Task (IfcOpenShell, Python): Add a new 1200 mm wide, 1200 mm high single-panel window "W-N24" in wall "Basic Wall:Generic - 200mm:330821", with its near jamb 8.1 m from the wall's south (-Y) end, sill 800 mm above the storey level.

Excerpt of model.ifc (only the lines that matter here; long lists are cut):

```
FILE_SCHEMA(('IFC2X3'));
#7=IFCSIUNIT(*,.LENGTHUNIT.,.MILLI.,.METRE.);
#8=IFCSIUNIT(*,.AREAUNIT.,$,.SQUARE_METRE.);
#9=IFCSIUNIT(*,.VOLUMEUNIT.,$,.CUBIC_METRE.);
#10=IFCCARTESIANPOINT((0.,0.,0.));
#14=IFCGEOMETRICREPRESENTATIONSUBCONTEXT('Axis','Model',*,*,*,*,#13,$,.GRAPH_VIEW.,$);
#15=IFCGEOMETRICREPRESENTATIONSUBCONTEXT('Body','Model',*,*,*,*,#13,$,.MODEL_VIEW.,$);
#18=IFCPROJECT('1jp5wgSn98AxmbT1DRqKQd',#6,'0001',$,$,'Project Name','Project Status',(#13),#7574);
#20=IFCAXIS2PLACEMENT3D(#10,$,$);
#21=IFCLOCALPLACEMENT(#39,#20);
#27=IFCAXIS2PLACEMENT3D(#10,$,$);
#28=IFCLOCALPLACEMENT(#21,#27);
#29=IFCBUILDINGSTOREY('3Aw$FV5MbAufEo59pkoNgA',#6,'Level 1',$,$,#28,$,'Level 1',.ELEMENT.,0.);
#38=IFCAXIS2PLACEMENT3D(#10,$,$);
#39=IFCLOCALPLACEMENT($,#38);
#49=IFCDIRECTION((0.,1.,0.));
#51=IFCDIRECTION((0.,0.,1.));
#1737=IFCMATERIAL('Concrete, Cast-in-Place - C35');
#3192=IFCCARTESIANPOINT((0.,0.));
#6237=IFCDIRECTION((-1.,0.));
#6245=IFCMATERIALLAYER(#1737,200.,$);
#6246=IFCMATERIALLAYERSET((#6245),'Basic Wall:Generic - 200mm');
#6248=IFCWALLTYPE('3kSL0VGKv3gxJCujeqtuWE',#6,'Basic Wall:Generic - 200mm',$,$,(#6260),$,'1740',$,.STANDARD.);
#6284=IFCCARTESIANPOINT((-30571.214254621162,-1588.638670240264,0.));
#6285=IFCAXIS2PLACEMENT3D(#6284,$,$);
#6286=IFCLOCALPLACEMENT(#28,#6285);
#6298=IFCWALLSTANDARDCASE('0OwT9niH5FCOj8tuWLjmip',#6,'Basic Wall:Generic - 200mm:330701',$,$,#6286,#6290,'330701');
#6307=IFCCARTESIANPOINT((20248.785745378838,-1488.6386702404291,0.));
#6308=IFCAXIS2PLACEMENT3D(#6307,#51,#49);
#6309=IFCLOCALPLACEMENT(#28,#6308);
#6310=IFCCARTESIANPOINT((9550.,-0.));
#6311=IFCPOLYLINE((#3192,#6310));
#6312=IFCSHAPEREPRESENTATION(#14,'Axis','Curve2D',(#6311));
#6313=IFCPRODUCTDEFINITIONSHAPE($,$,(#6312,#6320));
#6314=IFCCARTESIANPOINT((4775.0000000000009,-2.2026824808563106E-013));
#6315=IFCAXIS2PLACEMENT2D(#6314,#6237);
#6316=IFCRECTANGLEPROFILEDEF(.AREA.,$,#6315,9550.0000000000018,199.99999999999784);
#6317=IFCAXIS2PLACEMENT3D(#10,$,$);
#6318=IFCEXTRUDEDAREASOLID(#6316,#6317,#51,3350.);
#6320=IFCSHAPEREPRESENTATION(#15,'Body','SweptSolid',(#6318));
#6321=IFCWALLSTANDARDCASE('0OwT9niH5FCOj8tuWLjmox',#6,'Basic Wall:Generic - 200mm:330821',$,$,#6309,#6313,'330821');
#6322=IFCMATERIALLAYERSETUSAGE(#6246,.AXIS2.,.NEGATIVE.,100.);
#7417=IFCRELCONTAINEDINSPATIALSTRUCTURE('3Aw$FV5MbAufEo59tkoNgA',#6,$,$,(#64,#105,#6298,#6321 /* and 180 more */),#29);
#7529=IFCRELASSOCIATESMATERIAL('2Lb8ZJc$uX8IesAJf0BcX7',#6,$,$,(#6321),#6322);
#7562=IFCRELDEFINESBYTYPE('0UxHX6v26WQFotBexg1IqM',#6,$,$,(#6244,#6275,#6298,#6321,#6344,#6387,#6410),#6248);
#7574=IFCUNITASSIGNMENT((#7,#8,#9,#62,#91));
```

```python
import numpy as np
import ifcopenshell
import ifcopenshell.api.feature
import ifcopenshell.api.geometry
import ifcopenshell.api.root
import ifcopenshell.api.spatial
import ifcopenshell.api.type
import ifcopenshell.geom
import ifcopenshell.util.element
import ifcopenshell.util.placement
import ifcopenshell.util.representation
import ifcopenshell.util.shape
import ifcopenshell.util.unit

model = ifcopenshell.open("model.ifc")
unit_scale = ifcopenshell.util.unit.calculate_unit_scale(model)
settings = ifcopenshell.geom.settings()


def volume(element):
    """Net volume in cubic metres, openings subtracted."""
    shape = ifcopenshell.geom.create_shape(settings, element)
    return ifcopenshell.util.shape.get_volume(shape.geometry)


wall = model.by_guid("0OwT9niH5FCOj8tuWLjmox")
storey = ifcopenshell.util.element.get_container(wall, ifc_class="IfcBuildingStorey")
context = ifcopenshell.util.representation.get_context(model, "Model", "Body", "MODEL_VIEW")
before = volume(wall)

width, height, from_end, sill = 1.2, 1.2, 8.1, 0.8  # metres

# The wall runs along its own X axis, and the end named is its -X end.
wall_shape = ifcopenshell.geom.create_shape(settings, wall)
x, y, z = ifcopenshell.util.shape.get_vertices(wall_shape.geometry).T
start = x.min() + from_end
face, thickness = float(y.min()), float(y.max() - y.min())
wall_matrix = ifcopenshell.util.placement.get_local_placement(wall.ObjectPlacement)
level = ifcopenshell.util.placement.get_local_placement(storey.ObjectPlacement)[2, 3]


def in_wall(x, y):
    """Placement at x, y metres in the wall's axes, at sill height."""
    matrix = wall_matrix.copy()
    matrix[:, 3] = wall_matrix @ np.array([x / unit_scale, y / unit_scale, 0.0, 1.0])
    matrix[2, 3] = level + sill / unit_scale
    return matrix


# Opening: a box that overshoots both wall faces by 50 mm.
opening = ifcopenshell.api.root.create_entity(model, ifc_class="IfcOpeningElement")
box = ifcopenshell.api.geometry.add_wall_representation(
    model, context=context, length=width, height=height, thickness=thickness + 0.1
)
ifcopenshell.api.geometry.assign_representation(model, product=opening, representation=box)
ifcopenshell.api.geometry.edit_object_placement(model, product=opening, matrix=in_wall(start, face - 0.05), is_si=False)
ifcopenshell.api.feature.add_feature(model, feature=opening, element=wall)

window = ifcopenshell.api.root.create_entity(model, ifc_class="IfcWindow", name="W-N24")
window.OverallWidth, window.OverallHeight = width / unit_scale, height / unit_scale
body = ifcopenshell.api.geometry.add_window_representation(
    model,
    context=context,
    overall_width=window.OverallWidth,
    overall_height=window.OverallHeight,
    partition_type="SINGLE_PANEL",
)
ifcopenshell.api.geometry.assign_representation(model, product=window, representation=body)
ifcopenshell.api.spatial.assign_container(model, products=[window], relating_structure=storey)
fills = ifcopenshell.api.feature.add_filling(model, opening=opening, element=window)
fills.OwnerHistory = window.OwnerHistory  # required in IFC2X3

# IFC2X3 keeps the operation on the window style.
style = ifcopenshell.api.root.create_entity(model, ifc_class="IfcWindowStyle", name="W-N24")
style.OperationType, style.ConstructionType = "SINGLE_PANEL", "NOTDEFINED"
style.ParameterTakesPrecedence = style.Sizeable = False
ifcopenshell.api.type.assign_type(model, related_objects=[window], relating_type=style)

# Centre the window in the wall's thickness.
ifcopenshell.api.geometry.edit_object_placement(model, product=window, matrix=in_wall(start, face), is_si=False)
window_shape = ifcopenshell.geom.create_shape(settings, window)
depth = ifcopenshell.util.shape.get_vertices(window_shape.geometry)[:, 1]
offset = face + thickness / 2 - (depth.min() + depth.max()) / 2
ifcopenshell.api.geometry.edit_object_placement(model, product=window, matrix=in_wall(start, offset), is_si=False)

after = volume(wall)

print(f"wall volume {before:.3f} -> {after:.3f} m3")

model.write("model_updated.ifc")
```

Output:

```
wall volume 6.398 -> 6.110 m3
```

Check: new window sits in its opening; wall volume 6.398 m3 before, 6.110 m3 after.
